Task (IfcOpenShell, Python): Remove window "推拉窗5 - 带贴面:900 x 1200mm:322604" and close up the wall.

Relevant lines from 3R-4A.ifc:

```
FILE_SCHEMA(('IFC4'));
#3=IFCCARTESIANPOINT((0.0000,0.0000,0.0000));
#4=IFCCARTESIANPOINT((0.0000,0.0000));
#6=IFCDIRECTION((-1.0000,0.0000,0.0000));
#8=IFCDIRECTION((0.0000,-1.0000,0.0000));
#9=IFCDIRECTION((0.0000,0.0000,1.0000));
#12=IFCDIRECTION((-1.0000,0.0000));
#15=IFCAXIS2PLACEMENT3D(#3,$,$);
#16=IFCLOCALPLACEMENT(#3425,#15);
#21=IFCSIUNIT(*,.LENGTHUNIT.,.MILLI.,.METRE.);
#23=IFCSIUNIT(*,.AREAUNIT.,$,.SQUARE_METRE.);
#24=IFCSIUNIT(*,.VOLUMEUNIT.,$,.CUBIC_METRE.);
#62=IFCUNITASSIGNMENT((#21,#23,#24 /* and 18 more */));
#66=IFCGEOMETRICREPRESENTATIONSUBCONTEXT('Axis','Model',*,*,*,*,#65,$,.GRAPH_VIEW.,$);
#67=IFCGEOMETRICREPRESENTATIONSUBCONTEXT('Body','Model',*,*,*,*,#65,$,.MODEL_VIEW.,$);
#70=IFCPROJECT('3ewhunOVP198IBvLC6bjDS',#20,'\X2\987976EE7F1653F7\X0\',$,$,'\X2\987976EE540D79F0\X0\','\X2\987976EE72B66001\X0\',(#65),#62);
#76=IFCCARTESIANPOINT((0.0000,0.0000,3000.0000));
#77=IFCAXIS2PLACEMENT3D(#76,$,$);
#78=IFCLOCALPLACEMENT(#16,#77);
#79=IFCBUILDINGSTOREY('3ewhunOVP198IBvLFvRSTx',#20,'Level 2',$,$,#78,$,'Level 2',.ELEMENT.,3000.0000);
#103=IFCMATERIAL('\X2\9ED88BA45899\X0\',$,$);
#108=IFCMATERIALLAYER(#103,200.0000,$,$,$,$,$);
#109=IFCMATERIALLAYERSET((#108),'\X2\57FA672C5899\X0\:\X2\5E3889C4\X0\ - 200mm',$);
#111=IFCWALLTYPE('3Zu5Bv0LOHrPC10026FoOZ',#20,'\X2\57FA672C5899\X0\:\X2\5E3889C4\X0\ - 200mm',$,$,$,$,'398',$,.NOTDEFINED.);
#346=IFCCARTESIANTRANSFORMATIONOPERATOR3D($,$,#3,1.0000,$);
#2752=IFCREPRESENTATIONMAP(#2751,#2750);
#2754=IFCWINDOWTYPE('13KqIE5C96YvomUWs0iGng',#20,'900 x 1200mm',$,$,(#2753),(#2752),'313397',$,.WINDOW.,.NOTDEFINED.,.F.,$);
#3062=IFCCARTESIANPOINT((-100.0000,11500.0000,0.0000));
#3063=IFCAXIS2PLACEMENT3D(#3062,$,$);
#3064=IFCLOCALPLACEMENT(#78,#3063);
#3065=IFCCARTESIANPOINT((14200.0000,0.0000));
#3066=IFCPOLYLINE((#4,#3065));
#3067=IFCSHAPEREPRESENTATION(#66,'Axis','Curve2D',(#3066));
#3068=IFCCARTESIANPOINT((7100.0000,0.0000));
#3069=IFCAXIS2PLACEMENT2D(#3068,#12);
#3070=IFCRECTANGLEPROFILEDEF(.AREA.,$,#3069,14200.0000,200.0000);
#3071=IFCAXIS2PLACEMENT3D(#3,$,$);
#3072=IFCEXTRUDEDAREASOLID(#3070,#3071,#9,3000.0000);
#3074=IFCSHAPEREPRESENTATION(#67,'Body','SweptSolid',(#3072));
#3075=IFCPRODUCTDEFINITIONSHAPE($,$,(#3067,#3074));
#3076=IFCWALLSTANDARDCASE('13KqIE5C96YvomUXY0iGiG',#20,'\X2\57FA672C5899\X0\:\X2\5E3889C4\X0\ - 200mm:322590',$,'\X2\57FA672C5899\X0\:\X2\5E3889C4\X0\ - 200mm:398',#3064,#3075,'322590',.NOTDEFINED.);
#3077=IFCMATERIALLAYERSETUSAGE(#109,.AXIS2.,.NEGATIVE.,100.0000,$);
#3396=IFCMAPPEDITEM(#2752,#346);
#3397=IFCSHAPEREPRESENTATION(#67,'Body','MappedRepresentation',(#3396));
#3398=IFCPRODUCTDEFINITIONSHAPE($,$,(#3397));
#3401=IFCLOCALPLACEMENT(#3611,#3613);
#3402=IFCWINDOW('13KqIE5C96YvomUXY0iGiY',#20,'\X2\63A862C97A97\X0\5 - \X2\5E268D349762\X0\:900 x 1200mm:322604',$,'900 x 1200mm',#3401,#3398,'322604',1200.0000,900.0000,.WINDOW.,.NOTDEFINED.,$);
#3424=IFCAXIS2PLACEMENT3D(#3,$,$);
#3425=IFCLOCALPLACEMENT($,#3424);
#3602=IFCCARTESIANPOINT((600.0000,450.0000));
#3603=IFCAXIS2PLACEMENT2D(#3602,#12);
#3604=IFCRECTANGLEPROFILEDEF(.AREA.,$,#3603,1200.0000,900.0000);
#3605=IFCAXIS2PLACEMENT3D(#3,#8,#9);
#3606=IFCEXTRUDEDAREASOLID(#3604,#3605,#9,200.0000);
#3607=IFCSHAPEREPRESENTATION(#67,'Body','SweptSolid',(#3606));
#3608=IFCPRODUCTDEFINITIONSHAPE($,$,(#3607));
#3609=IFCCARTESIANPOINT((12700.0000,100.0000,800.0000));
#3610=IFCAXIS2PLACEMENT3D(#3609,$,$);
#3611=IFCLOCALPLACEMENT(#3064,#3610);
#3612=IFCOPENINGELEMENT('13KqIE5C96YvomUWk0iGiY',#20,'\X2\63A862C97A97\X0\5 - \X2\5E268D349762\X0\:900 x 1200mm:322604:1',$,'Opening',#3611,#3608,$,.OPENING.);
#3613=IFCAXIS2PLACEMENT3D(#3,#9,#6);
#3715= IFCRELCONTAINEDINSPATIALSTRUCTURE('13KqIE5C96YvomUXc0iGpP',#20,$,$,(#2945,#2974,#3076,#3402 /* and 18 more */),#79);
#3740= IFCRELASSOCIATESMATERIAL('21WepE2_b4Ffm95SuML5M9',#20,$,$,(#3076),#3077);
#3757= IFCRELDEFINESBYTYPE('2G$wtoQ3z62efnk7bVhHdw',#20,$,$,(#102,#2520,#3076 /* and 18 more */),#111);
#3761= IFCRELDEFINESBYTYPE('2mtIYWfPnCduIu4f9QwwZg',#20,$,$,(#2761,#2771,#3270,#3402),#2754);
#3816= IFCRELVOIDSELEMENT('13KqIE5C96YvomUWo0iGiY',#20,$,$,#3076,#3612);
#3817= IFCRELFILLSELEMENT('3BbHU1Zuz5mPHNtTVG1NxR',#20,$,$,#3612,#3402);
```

```python
import ifcopenshell
import ifcopenshell.api.feature
import ifcopenshell.api.root
import ifcopenshell.geom
import ifcopenshell.util.shape

model = ifcopenshell.open("3R-4A.ifc")
settings = ifcopenshell.geom.settings()


def volume(element):
    """Net volume in cubic metres, openings subtracted."""
    shape = ifcopenshell.geom.create_shape(settings, element)
    return ifcopenshell.util.shape.get_volume(shape.geometry)


window = model.by_id(3402)
opening = window.FillsVoids[0].RelatingOpeningElement
wall = opening.VoidsElements[0].RelatingBuildingElement
before = volume(wall)

ifcopenshell.api.root.remove_product(model, product=window)
ifcopenshell.api.feature.remove_feature(model, feature=opening)

after = volume(wall)

print(f"wall volume {before:.3f} -> {after:.3f} m3")

model.write("3R-4A_edited.ifc")
```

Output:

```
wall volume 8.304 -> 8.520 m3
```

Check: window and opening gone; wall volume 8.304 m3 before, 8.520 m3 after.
